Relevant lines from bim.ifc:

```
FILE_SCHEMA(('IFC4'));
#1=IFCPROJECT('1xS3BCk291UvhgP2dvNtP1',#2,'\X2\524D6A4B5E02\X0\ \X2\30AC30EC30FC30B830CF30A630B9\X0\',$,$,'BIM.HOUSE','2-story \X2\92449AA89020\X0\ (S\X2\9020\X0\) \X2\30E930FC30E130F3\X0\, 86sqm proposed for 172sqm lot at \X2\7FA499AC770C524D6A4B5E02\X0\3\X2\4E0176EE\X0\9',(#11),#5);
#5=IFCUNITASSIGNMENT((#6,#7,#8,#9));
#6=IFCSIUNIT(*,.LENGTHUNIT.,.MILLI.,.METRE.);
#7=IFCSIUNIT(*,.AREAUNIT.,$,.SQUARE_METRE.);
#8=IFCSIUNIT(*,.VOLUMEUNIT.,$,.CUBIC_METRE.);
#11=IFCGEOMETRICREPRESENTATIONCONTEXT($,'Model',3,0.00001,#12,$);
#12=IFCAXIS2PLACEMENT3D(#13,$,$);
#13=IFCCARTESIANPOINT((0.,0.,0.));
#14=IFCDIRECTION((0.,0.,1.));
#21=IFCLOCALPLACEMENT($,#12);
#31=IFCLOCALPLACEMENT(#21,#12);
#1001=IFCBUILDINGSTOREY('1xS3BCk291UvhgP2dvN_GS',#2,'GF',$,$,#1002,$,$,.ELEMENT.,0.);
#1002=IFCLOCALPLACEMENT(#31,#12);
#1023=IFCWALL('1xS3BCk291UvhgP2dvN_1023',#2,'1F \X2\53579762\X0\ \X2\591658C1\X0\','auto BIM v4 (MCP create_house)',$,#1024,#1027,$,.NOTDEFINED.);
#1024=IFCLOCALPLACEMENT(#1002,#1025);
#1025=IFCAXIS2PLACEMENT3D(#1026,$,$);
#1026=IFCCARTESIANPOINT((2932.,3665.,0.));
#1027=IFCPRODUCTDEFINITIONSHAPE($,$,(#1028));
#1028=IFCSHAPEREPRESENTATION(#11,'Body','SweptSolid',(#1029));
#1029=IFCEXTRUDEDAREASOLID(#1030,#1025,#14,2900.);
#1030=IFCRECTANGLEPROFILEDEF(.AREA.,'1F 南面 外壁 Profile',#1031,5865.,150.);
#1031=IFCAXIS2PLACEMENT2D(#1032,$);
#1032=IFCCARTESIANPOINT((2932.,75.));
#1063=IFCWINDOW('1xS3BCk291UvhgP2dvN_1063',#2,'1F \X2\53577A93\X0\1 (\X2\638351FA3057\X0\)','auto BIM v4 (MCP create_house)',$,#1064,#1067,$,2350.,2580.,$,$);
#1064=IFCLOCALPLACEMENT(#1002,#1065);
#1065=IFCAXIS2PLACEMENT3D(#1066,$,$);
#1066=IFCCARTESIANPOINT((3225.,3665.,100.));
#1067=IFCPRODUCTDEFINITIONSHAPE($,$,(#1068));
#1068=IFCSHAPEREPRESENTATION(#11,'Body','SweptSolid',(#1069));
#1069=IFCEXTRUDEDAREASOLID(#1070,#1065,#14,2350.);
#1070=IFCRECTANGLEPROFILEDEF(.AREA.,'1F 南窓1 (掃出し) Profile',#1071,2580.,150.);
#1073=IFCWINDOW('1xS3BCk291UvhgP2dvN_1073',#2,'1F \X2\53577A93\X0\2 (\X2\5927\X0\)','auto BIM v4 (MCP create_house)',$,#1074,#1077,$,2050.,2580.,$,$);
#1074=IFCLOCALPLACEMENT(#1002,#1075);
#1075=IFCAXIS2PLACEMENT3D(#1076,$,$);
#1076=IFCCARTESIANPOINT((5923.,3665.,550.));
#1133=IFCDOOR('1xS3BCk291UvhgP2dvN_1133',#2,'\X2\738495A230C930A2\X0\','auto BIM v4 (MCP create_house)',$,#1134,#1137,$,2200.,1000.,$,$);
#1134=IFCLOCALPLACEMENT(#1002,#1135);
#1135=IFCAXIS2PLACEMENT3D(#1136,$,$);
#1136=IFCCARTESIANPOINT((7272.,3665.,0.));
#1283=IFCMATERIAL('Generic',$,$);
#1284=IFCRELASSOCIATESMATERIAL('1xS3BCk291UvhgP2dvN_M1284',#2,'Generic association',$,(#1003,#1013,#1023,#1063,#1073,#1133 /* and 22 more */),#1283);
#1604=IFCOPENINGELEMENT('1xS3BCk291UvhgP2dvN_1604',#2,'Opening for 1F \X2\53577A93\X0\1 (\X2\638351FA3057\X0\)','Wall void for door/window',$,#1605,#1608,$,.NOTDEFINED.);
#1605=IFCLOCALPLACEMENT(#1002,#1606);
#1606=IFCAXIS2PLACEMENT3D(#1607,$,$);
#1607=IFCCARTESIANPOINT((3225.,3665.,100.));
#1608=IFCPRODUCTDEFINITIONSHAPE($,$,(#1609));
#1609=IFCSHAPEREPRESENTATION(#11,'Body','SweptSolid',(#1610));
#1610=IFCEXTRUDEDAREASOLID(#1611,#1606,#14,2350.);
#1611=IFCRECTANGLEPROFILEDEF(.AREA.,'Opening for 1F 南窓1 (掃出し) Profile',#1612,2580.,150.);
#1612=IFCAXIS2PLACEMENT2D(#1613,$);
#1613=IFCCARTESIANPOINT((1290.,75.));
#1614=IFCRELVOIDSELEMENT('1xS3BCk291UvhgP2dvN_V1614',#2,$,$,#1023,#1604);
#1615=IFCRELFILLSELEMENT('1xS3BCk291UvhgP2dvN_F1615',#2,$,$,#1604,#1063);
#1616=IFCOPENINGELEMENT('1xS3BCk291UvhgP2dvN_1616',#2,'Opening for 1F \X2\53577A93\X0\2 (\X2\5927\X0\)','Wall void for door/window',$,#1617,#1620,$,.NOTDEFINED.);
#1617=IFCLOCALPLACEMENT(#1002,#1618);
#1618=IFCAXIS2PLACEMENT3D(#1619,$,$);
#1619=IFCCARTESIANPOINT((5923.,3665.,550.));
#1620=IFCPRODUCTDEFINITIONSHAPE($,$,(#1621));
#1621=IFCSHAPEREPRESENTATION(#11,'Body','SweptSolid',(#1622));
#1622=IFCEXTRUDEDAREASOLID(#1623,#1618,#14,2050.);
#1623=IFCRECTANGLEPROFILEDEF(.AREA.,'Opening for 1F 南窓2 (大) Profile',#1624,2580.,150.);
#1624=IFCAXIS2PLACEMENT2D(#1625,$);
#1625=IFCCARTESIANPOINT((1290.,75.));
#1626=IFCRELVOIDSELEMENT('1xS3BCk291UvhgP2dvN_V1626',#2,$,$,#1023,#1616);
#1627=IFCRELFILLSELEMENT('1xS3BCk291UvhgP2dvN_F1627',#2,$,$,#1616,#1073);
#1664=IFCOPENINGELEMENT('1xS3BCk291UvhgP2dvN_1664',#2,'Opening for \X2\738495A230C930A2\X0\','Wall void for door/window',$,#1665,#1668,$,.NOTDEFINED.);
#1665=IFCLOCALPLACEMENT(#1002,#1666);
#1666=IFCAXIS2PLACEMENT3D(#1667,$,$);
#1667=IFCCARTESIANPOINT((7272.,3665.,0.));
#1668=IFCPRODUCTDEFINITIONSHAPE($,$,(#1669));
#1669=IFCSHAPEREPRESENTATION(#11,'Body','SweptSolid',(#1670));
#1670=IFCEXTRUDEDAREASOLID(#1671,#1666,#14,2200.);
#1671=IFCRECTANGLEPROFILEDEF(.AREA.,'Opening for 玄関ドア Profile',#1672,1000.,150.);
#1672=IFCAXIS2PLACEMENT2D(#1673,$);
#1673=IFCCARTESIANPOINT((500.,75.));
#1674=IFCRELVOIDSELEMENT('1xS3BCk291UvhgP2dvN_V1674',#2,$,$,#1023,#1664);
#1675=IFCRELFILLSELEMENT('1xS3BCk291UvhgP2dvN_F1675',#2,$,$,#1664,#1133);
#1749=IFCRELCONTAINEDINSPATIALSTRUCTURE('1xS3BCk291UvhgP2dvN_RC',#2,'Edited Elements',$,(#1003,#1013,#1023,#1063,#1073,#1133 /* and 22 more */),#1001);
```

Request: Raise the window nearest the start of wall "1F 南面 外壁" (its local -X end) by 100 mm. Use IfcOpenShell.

```python
import numpy as np
import ifcopenshell
import ifcopenshell.api.geometry
import ifcopenshell.util.placement
import ifcopenshell.util.unit

model = ifcopenshell.open("bim.ifc")
unit_scale = ifcopenshell.util.unit.calculate_unit_scale(model)

window = model.by_guid("1xS3BCk291UvhgP2dvN_1063")
opening = window.FillsVoids[0].RelatingOpeningElement
dz = 100.0

shift = np.array([0.0, 0.0, dz])
# The window is not placed relative to its opening, so move both.
for product in (opening, window):
    matrix = ifcopenshell.util.placement.get_local_placement(product.ObjectPlacement)
    matrix[:3, 3] += shift
    ifcopenshell.api.geometry.edit_object_placement(model, product=product, matrix=matrix, is_si=False)

print(f"moved by {dz * unit_scale:+.3f} m")

model.write("bim_updated.ifc")
```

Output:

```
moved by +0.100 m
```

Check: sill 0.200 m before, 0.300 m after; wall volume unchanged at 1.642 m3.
